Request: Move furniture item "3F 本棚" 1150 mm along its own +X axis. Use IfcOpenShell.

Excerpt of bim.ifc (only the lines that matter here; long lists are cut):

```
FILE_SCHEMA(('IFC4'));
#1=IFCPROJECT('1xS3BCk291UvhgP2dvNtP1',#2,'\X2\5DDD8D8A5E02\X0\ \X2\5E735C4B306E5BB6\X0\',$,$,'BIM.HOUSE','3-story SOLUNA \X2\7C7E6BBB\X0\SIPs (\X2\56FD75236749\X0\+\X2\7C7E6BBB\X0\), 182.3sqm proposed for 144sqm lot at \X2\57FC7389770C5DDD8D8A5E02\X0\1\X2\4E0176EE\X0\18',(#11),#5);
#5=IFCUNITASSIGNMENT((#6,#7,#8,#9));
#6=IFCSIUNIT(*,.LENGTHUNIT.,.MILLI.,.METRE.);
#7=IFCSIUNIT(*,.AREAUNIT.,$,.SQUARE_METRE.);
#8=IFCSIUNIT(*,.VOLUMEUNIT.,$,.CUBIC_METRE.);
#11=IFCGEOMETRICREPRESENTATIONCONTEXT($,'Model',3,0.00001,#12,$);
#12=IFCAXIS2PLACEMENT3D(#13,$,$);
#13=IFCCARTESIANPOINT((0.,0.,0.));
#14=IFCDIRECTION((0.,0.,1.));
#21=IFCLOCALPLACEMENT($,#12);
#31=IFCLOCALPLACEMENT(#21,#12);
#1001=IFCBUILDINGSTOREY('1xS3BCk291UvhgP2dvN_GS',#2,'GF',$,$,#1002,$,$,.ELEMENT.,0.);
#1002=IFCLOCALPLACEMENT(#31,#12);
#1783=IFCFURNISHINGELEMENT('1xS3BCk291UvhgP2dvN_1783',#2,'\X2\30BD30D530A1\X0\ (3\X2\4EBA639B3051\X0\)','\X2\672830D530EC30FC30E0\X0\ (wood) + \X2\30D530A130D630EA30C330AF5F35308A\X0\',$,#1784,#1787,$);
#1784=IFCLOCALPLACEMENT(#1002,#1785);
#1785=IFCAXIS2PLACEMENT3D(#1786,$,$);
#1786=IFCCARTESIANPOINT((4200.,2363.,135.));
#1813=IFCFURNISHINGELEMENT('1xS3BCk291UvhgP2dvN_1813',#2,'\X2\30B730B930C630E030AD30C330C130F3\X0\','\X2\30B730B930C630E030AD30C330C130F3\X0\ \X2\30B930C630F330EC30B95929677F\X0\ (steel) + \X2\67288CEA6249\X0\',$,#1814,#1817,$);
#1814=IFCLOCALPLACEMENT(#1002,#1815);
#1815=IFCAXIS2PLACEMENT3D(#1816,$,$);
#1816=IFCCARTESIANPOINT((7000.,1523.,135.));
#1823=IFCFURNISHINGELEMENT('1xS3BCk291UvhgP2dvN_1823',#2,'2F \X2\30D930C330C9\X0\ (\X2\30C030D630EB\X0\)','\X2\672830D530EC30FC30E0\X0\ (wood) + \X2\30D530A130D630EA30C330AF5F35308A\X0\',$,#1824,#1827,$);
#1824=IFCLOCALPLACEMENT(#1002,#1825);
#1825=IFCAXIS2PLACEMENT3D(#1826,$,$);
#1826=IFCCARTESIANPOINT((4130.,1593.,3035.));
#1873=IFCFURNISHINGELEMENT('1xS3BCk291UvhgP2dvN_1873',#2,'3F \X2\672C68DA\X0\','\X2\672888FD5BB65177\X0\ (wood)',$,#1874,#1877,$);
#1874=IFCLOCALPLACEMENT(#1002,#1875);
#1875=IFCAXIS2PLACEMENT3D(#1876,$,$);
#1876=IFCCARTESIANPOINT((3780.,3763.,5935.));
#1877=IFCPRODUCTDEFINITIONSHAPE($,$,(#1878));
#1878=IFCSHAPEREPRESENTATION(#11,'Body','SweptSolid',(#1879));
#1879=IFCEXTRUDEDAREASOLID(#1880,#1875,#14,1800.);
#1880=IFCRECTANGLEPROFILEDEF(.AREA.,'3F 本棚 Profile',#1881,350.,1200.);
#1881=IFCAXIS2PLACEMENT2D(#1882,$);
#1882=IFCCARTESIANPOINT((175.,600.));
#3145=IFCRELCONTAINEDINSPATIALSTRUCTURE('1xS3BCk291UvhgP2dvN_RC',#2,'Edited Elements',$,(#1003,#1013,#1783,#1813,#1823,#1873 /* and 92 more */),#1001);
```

```python
import ifcopenshell
import ifcopenshell.api.geometry
import ifcopenshell.util.placement
import ifcopenshell.util.unit

model = ifcopenshell.open("bim.ifc")
unit_scale = ifcopenshell.util.unit.calculate_unit_scale(model)

item = model.by_guid("1xS3BCk291UvhgP2dvN_1873")
matrix = ifcopenshell.util.placement.get_local_placement(item.ObjectPlacement)
matrix[:3, 3] += matrix[:3, 0] * 1.15 / unit_scale
ifcopenshell.api.geometry.edit_object_placement(model, product=item, matrix=matrix, is_si=False)

print(ifcopenshell.util.placement.get_local_placement(item.ObjectPlacement).round(3) + 0.0)

model.write("bim_v2.ifc")
```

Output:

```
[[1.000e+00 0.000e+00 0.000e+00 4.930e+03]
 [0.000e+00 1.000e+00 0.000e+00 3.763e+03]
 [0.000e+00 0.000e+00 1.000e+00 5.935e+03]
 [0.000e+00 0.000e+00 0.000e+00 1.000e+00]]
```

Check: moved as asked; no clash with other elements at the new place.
